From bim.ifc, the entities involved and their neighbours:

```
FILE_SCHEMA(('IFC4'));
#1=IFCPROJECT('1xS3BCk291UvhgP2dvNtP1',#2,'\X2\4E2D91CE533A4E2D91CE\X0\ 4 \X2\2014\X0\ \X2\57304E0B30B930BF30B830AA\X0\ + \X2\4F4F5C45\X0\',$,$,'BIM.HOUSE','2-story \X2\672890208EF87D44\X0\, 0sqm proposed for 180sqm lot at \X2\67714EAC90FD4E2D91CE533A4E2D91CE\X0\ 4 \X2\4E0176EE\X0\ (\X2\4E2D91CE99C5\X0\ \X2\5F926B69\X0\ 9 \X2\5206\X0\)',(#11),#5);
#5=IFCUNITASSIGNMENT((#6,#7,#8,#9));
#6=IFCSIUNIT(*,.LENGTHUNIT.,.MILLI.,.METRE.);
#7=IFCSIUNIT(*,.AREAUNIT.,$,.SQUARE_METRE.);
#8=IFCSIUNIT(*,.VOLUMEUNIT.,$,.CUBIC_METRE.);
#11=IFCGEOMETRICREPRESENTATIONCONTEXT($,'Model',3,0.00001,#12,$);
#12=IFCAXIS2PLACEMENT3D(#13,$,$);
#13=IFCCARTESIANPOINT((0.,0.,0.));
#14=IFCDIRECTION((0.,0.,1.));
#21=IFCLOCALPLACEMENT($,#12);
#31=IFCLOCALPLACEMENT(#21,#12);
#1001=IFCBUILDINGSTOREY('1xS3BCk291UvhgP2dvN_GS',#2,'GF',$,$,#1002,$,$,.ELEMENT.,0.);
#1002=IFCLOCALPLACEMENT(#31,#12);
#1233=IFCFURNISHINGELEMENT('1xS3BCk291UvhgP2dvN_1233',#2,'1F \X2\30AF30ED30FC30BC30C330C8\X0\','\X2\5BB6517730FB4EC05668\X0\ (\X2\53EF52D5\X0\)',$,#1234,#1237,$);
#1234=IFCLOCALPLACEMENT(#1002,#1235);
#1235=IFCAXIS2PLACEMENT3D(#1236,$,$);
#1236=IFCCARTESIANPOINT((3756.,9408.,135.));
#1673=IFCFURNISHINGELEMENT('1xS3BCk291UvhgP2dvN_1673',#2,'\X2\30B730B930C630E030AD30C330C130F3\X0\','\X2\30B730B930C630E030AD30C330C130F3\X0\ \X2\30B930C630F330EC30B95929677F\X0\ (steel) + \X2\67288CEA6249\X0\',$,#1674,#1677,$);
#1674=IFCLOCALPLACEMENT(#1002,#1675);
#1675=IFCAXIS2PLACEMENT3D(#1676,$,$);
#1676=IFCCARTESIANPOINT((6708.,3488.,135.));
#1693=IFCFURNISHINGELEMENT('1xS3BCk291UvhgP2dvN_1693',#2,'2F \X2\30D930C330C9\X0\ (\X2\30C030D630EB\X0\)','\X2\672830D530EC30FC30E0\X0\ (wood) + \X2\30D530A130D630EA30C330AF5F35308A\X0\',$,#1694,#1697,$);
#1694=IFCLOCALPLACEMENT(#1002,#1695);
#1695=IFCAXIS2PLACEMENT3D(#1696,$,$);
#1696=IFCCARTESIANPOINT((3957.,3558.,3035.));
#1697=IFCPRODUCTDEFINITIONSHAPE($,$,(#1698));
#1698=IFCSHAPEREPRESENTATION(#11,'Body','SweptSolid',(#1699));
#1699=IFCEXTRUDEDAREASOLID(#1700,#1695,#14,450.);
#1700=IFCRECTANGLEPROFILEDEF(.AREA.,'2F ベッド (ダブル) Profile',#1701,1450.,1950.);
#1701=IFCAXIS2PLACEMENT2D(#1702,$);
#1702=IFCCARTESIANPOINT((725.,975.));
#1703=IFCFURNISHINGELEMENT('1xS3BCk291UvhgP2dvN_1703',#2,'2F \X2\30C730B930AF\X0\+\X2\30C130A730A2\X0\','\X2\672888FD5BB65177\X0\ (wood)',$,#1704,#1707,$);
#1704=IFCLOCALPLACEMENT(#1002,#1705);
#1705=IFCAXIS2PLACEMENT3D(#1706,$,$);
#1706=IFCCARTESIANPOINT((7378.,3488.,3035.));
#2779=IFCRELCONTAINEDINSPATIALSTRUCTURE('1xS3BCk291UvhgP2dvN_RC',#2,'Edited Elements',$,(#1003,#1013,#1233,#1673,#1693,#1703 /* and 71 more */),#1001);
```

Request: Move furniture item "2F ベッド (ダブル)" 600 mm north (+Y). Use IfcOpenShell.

```python
import ifcopenshell
import ifcopenshell.api.geometry
import ifcopenshell.util.placement

model = ifcopenshell.open("bim.ifc")

item = model.by_guid("1xS3BCk291UvhgP2dvN_1693")
matrix = ifcopenshell.util.placement.get_local_placement(item.ObjectPlacement)
matrix[1, 3] += 600.0
ifcopenshell.api.geometry.edit_object_placement(model, product=item, matrix=matrix, is_si=False)

print(ifcopenshell.util.placement.get_local_placement(item.ObjectPlacement).round(3) + 0.0)

model.write("bim_edited.ifc")
```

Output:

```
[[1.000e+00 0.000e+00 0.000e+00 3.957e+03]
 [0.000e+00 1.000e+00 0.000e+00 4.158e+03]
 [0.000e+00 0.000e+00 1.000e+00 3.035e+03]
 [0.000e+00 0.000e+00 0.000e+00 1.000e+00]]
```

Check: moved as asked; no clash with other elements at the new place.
